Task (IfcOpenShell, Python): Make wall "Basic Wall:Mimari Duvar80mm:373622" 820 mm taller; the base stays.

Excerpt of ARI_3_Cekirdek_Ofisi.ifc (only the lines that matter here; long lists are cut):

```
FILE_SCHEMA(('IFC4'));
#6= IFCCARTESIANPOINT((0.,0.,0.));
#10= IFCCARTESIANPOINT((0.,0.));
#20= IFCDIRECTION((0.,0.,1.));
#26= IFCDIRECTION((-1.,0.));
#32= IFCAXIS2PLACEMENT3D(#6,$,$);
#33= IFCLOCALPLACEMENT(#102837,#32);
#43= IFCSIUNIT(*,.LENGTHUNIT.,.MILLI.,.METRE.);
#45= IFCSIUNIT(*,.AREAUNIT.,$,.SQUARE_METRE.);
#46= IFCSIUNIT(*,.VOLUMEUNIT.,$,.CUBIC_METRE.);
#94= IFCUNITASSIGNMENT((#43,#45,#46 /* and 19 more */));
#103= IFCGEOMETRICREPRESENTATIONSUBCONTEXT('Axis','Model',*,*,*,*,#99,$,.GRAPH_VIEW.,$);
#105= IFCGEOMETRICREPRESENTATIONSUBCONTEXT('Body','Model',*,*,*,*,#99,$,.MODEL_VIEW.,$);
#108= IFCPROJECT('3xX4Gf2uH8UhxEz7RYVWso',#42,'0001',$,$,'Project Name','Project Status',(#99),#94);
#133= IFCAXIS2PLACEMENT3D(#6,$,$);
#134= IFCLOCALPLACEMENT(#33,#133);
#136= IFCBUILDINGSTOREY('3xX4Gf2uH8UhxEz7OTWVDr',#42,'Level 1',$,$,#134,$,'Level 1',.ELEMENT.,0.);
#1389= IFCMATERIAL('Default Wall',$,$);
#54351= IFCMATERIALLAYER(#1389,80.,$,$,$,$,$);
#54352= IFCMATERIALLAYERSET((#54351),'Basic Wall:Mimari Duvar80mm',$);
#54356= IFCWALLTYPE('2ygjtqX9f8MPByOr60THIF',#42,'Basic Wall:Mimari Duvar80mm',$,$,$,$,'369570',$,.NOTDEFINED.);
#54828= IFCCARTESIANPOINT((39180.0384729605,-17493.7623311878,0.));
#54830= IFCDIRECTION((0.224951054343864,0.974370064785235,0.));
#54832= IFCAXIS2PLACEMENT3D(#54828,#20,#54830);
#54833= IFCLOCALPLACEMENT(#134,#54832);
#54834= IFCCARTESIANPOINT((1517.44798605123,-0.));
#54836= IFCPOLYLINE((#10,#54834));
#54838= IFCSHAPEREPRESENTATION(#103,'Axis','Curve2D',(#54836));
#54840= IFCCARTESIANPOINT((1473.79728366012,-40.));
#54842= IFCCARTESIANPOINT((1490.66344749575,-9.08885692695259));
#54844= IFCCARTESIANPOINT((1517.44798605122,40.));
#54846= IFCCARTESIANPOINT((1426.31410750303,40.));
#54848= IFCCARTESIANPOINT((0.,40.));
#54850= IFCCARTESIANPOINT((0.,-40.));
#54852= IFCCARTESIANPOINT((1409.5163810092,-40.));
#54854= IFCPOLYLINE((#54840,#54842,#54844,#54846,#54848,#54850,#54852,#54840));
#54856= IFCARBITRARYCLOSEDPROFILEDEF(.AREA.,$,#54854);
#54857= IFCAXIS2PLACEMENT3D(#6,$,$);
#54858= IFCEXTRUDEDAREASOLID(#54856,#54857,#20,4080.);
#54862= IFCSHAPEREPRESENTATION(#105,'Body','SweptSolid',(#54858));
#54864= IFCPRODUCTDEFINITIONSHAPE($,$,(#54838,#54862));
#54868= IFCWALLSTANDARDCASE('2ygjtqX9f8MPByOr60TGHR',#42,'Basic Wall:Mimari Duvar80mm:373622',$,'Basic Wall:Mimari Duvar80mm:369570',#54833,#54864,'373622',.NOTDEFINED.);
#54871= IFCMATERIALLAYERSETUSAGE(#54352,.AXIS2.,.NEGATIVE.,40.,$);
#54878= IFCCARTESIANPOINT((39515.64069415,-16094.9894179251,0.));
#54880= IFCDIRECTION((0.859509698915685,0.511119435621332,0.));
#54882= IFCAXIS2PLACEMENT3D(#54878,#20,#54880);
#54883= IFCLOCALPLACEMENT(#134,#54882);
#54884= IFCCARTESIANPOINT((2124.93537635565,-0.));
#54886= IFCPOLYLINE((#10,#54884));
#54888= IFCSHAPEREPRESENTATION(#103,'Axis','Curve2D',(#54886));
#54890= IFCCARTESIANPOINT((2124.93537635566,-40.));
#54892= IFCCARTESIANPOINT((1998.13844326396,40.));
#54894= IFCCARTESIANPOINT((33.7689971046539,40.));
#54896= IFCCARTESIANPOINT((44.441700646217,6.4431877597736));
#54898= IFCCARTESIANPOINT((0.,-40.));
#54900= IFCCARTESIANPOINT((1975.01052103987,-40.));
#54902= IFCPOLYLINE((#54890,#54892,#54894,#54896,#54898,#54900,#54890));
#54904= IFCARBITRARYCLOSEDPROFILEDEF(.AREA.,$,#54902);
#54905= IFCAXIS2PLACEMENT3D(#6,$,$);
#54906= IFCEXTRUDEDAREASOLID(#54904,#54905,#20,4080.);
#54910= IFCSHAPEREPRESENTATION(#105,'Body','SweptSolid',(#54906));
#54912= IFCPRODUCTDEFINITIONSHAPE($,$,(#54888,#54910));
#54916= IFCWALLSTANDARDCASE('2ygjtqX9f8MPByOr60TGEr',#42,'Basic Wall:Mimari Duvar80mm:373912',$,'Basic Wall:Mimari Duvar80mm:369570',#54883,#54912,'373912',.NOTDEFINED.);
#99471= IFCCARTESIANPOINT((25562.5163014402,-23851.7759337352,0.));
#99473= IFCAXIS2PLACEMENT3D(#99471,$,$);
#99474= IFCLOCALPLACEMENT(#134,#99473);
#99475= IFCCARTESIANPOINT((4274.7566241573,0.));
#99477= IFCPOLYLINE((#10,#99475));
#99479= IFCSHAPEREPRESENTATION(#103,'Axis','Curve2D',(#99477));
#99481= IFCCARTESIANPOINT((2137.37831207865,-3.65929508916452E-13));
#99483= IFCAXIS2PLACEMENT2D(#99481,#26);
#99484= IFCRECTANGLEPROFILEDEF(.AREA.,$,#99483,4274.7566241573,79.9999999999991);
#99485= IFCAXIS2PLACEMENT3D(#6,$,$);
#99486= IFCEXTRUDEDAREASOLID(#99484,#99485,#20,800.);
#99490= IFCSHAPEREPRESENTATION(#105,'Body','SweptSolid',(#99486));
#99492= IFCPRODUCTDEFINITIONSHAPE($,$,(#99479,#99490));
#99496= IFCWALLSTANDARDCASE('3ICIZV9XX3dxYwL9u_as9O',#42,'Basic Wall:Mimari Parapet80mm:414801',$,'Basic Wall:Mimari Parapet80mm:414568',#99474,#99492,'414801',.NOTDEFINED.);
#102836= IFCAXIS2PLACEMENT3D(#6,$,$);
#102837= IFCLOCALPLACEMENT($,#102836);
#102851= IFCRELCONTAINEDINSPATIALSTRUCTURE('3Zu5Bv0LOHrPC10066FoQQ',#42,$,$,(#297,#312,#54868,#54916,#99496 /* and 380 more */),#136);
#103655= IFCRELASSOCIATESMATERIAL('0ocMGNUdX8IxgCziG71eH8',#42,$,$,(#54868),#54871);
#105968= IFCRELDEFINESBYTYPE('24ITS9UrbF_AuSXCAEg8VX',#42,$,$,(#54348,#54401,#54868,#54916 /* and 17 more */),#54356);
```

```python
import ifcopenshell
import ifcopenshell.geom
import ifcopenshell.util.representation
import ifcopenshell.util.shape

model = ifcopenshell.open("ARI_3_Cekirdek_Ofisi.ifc")
settings = ifcopenshell.geom.settings()


def volume(element):
    """Net volume in cubic metres, openings subtracted."""
    shape = ifcopenshell.geom.create_shape(settings, element)
    return ifcopenshell.util.shape.get_volume(shape.geometry)


wall = model.by_guid("2ygjtqX9f8MPByOr60TGHR")
before = volume(wall)

body = ifcopenshell.util.representation.get_representation(wall, "Model", "Body")
solid = body.Items[0]
old_height = solid.Depth
solid.Depth += 820.0
after = volume(wall)

print(f"height {old_height:g} -> {solid.Depth:g}, volume {before:.3f} -> {after:.3f} m3")

model.write("ARI_3_Cekirdek_Ofisi_updated.ifc")
```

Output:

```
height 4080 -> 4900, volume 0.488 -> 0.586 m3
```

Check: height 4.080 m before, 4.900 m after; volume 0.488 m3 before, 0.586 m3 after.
